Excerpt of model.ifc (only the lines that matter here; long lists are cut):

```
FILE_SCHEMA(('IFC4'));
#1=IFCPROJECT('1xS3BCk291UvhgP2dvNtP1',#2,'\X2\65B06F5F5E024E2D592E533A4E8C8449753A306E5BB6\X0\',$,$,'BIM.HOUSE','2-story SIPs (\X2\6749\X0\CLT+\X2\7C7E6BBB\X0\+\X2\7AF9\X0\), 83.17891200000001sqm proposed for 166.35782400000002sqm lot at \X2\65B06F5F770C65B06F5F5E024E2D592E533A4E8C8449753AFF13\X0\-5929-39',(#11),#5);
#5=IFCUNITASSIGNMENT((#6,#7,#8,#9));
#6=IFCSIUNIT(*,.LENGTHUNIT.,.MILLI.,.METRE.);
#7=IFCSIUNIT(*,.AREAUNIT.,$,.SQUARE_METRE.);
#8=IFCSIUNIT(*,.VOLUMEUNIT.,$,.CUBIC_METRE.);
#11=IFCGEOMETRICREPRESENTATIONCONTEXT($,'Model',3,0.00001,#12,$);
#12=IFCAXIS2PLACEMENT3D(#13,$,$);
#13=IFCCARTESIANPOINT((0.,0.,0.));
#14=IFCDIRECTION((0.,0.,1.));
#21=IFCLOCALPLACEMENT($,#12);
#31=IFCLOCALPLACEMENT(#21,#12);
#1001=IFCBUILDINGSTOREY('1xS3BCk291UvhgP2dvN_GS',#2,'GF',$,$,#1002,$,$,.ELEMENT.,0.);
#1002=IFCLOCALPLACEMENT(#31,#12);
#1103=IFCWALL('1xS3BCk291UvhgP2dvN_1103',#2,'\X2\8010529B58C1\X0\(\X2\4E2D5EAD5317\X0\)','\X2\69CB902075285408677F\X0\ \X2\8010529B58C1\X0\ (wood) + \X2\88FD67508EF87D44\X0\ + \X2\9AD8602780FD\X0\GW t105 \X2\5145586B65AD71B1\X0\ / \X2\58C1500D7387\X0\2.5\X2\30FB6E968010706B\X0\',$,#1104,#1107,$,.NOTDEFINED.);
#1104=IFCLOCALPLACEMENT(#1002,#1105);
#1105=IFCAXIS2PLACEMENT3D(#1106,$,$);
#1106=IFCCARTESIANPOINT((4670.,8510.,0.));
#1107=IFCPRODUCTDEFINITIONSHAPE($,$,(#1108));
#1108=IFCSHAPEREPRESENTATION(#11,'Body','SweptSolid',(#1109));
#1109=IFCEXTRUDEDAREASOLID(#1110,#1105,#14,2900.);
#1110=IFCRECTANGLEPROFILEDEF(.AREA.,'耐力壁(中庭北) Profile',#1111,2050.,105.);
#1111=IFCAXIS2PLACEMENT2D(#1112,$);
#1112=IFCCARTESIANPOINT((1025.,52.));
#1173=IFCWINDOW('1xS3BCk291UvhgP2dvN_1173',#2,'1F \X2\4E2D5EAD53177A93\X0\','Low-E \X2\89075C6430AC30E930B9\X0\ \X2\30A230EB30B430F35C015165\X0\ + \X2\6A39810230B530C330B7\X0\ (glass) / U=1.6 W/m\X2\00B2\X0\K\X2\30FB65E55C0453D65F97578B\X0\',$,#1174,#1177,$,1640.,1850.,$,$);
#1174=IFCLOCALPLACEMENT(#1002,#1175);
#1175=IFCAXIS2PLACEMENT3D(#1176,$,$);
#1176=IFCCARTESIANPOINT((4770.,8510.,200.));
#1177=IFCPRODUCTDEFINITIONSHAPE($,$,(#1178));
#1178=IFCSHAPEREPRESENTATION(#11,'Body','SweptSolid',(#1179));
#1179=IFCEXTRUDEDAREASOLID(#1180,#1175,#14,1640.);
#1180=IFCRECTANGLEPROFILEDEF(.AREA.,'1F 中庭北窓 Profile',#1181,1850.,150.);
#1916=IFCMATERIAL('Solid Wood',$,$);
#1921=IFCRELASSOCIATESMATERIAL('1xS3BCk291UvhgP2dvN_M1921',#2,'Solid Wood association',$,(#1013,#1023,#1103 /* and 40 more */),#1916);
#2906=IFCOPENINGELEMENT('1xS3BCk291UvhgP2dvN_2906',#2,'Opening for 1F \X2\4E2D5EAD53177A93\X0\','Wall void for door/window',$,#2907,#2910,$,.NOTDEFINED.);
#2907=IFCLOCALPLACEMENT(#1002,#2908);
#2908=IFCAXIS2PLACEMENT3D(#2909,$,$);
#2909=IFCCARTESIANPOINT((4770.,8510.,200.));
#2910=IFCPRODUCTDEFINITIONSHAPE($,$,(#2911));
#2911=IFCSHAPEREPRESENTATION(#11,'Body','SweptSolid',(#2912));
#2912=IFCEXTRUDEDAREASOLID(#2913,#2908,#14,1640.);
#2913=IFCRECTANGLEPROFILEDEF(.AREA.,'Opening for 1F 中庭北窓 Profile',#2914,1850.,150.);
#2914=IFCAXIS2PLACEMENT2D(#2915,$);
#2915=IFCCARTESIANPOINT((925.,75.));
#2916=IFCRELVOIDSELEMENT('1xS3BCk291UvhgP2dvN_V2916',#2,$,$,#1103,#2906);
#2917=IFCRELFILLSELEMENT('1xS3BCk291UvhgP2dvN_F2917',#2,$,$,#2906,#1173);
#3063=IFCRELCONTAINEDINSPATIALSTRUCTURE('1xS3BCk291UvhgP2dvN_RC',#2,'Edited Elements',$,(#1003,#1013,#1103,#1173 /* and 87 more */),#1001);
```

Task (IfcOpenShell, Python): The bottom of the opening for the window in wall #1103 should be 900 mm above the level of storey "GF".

```python
import numpy as np
import ifcopenshell
import ifcopenshell.api.geometry
import ifcopenshell.geom
import ifcopenshell.util.element
import ifcopenshell.util.placement
import ifcopenshell.util.shape
import ifcopenshell.util.unit

model = ifcopenshell.open("model.ifc")
unit_scale = ifcopenshell.util.unit.calculate_unit_scale(model)

window = model.by_guid("1xS3BCk291UvhgP2dvN_1173")
opening = window.FillsVoids[0].RelatingOpeningElement
storey = ifcopenshell.util.element.get_container(window, ifc_class="IfcBuildingStorey")
level = ifcopenshell.util.placement.get_local_placement(storey.ObjectPlacement)[2, 3]

# The opening's origin need not be at the sill, so measure its lowest point.
shape = ifcopenshell.geom.create_shape(ifcopenshell.geom.settings(), opening)
bottom = ifcopenshell.util.shape.get_shape_bottom_elevation(shape, shape.geometry) / unit_scale
dz = level + 900.0 - bottom

shift = np.array([0.0, 0.0, dz])
# The window is not placed relative to its opening, so move both.
for product in (opening, window):
    matrix = ifcopenshell.util.placement.get_local_placement(product.ObjectPlacement)
    matrix[:3, 3] += shift
    ifcopenshell.api.geometry.edit_object_placement(model, product=product, matrix=matrix, is_si=False)

print(f"moved by {dz * unit_scale:+.3f} m")

model.write("model_updated.ifc")
```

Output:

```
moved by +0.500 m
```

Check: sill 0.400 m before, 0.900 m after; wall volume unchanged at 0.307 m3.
